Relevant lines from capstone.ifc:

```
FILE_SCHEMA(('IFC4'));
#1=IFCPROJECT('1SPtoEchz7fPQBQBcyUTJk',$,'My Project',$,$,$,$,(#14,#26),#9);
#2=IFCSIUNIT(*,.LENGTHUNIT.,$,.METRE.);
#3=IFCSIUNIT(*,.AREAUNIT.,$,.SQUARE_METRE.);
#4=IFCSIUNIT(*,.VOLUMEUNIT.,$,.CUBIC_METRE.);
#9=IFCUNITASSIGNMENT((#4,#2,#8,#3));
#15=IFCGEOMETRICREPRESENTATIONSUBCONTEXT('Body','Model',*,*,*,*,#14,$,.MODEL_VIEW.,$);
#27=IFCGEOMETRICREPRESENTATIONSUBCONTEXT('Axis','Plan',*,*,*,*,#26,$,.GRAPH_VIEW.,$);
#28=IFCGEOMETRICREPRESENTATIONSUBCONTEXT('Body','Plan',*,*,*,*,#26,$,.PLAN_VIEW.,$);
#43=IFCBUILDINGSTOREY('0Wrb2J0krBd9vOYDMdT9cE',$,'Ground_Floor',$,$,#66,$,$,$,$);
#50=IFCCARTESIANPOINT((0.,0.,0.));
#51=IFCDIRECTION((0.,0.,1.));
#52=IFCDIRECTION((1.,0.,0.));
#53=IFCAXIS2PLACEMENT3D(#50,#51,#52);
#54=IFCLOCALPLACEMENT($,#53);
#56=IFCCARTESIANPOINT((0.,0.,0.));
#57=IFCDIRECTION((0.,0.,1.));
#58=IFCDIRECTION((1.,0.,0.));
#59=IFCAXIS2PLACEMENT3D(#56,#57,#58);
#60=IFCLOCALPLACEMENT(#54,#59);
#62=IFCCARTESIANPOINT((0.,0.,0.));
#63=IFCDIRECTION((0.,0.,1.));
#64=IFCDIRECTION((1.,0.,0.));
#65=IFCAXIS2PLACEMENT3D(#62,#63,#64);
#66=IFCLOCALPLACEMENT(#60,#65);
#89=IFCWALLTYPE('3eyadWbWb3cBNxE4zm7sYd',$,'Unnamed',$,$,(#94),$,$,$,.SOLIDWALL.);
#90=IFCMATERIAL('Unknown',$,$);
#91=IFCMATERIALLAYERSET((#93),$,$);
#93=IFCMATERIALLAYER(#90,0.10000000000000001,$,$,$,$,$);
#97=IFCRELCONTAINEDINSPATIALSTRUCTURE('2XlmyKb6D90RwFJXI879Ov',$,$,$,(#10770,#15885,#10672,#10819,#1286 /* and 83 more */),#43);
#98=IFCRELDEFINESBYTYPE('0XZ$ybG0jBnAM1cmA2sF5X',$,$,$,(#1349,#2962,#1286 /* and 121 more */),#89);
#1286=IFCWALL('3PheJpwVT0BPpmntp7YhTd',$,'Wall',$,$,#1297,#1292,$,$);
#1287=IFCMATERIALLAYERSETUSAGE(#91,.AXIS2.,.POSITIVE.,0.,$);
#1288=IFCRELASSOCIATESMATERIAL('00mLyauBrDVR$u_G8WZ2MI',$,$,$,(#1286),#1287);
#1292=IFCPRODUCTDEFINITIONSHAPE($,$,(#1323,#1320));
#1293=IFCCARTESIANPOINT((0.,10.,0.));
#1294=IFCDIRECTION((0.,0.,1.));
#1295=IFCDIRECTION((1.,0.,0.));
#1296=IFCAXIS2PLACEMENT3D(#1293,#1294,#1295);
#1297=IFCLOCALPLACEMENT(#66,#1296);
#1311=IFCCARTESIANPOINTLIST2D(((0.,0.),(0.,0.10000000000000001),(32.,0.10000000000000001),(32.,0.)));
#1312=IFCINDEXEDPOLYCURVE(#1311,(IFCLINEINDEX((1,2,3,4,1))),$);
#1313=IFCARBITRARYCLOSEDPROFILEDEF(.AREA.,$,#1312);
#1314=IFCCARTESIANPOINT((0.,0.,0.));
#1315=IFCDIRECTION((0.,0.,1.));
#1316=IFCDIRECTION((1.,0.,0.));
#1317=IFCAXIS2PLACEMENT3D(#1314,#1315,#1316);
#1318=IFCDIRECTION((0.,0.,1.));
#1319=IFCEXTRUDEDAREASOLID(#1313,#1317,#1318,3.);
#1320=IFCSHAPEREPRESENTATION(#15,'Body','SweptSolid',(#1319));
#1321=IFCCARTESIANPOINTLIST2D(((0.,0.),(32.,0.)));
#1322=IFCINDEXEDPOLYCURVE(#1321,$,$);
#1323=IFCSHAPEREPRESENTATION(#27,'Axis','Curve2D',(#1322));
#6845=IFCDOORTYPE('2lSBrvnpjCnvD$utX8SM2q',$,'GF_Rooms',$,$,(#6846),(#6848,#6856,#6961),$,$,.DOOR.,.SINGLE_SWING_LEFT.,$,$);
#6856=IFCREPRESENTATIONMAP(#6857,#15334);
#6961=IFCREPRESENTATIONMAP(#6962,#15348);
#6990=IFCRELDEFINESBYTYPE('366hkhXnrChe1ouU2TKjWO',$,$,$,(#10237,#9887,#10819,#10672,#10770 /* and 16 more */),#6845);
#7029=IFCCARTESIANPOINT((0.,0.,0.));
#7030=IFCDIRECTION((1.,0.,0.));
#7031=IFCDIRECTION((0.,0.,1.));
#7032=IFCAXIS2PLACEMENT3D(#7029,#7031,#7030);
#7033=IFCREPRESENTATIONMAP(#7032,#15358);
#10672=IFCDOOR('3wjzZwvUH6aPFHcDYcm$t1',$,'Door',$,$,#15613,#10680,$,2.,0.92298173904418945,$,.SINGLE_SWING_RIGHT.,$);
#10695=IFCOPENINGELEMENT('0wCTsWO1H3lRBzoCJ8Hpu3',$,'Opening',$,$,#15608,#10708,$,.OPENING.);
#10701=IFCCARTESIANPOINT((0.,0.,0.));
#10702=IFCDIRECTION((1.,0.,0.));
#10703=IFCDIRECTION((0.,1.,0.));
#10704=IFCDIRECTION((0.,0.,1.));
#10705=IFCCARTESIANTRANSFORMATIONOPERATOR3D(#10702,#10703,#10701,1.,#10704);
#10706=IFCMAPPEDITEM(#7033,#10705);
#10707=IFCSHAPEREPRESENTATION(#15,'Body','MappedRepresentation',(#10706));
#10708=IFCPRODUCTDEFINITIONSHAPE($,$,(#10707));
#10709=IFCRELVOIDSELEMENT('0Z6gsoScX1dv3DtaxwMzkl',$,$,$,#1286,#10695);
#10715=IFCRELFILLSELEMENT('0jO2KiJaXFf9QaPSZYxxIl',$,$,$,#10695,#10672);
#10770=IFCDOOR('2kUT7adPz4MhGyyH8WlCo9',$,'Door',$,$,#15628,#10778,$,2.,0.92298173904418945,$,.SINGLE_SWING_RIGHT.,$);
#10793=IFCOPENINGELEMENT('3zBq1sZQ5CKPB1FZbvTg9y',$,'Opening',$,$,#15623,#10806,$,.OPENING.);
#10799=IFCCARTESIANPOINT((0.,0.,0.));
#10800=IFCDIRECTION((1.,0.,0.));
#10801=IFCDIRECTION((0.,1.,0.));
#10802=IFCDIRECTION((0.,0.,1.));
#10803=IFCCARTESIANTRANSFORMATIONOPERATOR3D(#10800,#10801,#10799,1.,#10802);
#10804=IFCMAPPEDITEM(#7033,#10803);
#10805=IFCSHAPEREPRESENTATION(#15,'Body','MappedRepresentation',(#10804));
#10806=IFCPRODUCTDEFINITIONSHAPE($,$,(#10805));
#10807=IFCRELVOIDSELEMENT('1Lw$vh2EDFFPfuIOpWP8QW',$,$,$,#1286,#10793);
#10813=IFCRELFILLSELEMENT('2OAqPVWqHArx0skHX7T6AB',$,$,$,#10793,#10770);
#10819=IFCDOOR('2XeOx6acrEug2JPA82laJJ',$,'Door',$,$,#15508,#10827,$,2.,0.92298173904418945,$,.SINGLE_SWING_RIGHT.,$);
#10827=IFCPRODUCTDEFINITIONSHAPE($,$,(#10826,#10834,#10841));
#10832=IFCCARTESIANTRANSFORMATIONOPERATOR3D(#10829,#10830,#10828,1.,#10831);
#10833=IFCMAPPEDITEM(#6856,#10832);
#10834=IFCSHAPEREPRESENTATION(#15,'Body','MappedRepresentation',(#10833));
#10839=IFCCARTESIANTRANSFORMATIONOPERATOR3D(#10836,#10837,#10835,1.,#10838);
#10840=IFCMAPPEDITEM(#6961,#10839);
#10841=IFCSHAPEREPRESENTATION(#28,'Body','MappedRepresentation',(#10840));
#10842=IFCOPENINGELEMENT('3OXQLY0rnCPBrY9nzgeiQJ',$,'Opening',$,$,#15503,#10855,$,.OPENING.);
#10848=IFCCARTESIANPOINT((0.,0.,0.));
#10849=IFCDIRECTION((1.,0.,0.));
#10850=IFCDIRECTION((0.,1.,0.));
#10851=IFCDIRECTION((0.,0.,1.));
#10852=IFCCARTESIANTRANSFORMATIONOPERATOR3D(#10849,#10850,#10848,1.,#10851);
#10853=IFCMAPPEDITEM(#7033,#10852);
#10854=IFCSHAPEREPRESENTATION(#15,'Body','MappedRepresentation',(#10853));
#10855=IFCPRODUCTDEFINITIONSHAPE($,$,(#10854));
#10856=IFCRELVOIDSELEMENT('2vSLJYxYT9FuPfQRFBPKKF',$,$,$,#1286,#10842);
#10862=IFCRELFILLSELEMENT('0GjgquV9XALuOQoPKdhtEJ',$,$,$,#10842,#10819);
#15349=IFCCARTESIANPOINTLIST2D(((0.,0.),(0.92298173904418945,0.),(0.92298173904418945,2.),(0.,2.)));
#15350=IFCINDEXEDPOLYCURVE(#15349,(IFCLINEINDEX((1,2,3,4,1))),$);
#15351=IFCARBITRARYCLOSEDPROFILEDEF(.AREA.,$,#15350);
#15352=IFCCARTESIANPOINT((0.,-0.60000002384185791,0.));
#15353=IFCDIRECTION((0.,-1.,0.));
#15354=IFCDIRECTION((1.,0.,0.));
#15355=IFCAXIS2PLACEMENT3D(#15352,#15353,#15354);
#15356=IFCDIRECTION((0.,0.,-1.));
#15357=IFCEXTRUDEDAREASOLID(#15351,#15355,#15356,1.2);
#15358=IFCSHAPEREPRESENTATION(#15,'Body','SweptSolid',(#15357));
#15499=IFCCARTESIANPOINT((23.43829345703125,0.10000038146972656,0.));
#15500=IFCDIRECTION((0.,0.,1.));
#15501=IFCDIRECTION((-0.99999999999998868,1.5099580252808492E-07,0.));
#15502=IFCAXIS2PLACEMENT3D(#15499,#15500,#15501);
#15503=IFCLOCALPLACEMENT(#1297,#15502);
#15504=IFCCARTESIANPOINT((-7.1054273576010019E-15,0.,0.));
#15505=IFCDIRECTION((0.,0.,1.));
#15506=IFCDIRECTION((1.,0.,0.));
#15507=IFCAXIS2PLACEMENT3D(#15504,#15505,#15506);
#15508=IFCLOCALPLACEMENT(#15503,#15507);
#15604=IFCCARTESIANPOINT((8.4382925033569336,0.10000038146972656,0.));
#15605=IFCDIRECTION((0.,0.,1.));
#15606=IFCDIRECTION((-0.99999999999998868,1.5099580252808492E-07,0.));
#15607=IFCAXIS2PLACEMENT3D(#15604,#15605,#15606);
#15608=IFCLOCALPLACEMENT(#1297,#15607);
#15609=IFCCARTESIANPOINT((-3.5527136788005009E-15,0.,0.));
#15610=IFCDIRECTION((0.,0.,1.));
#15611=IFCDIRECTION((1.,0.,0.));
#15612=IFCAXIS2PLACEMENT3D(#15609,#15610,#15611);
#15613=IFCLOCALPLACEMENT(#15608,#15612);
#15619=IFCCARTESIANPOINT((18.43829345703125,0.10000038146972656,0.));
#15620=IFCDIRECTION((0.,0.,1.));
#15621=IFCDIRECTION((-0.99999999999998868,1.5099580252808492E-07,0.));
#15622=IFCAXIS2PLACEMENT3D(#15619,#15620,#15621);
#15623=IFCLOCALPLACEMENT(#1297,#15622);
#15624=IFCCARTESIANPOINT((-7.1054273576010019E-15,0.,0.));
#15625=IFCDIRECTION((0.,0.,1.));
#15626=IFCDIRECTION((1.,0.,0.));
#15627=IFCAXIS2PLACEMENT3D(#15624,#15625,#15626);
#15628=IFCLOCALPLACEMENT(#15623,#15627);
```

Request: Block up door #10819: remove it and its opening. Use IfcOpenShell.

```python
import ifcopenshell
import ifcopenshell.api.feature
import ifcopenshell.api.root
import ifcopenshell.geom
import ifcopenshell.util.shape

model = ifcopenshell.open("capstone.ifc")
settings = ifcopenshell.geom.settings()


def volume(element):
    """Net volume in cubic metres, openings subtracted."""
    shape = ifcopenshell.geom.create_shape(settings, element)
    return ifcopenshell.util.shape.get_volume(shape.geometry)


door = model.by_guid("2XeOx6acrEug2JPA82laJJ")
opening = door.FillsVoids[0].RelatingOpeningElement
wall = opening.VoidsElements[0].RelatingBuildingElement
before = volume(wall)

ifcopenshell.api.root.remove_product(model, product=door)
ifcopenshell.api.feature.remove_feature(model, feature=opening)

after = volume(wall)

print(f"wall volume {before:.3f} -> {after:.3f} m3")

model.write("capstone_edited.ifc")
```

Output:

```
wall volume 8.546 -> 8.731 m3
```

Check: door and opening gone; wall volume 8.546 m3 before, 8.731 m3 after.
